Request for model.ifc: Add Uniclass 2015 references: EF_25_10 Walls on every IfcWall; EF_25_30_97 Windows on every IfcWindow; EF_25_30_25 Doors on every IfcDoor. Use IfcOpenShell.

First a look at what the model holds.

```python
import ifcopenshell

model = ifcopenshell.open("model.ifc")
print(model.schema)
print("classifications:", [c.Name for c in model.by_type("IfcClassification")])
for ifc_class in ("IfcDoor", "IfcRoof", "IfcStair", "IfcWall", "IfcWindow"):
    print(ifc_class, len(model.by_type(ifc_class)))
```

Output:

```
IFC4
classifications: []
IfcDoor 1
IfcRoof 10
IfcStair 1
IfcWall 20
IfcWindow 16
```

```python
import ifcopenshell
import ifcopenshell.api.classification

model = ifcopenshell.open("model.ifc")

system = ifcopenshell.api.classification.add_classification(model, classification="Uniclass 2015")

codes = {
    "IfcWall": ("EF_25_10", "Walls"),
    "IfcWindow": ("EF_25_30_97", "Windows"),
    "IfcDoor": ("EF_25_30_25", "Doors"),
}
for ifc_class, (code, name) in codes.items():
    products = model.by_type(ifc_class)
    ifcopenshell.api.classification.add_reference(
        model, products=products, classification=system, identification=code, name=name
    )
    print(code, len(products))

model.write("model_updated.ifc")
```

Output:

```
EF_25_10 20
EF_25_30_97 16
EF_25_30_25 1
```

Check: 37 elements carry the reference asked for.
